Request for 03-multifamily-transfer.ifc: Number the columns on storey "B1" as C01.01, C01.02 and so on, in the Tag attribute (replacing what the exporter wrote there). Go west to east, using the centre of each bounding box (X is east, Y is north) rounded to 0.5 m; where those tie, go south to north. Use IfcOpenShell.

First a look at what the model holds.

```python
import ifcopenshell
import ifcopenshell.util.element
import ifcopenshell.util.placement

model = ifcopenshell.open("03-multifamily-transfer.ifc")
print(model.schema)
storey = next(s for s in model.by_type("IfcBuildingStorey") if s.Name == "B1")
columns = [e for e in ifcopenshell.util.element.get_decomposition(storey) if e.is_a("IfcColumn")]
for e in sorted(columns, key=lambda e: e.id()):
    origin = ifcopenshell.util.placement.get_local_placement(e.ObjectPlacement)[:3, 3]
    print(e.id(), e.Tag, e.Name, origin.round(2) + 0.0, sep=" | ")
```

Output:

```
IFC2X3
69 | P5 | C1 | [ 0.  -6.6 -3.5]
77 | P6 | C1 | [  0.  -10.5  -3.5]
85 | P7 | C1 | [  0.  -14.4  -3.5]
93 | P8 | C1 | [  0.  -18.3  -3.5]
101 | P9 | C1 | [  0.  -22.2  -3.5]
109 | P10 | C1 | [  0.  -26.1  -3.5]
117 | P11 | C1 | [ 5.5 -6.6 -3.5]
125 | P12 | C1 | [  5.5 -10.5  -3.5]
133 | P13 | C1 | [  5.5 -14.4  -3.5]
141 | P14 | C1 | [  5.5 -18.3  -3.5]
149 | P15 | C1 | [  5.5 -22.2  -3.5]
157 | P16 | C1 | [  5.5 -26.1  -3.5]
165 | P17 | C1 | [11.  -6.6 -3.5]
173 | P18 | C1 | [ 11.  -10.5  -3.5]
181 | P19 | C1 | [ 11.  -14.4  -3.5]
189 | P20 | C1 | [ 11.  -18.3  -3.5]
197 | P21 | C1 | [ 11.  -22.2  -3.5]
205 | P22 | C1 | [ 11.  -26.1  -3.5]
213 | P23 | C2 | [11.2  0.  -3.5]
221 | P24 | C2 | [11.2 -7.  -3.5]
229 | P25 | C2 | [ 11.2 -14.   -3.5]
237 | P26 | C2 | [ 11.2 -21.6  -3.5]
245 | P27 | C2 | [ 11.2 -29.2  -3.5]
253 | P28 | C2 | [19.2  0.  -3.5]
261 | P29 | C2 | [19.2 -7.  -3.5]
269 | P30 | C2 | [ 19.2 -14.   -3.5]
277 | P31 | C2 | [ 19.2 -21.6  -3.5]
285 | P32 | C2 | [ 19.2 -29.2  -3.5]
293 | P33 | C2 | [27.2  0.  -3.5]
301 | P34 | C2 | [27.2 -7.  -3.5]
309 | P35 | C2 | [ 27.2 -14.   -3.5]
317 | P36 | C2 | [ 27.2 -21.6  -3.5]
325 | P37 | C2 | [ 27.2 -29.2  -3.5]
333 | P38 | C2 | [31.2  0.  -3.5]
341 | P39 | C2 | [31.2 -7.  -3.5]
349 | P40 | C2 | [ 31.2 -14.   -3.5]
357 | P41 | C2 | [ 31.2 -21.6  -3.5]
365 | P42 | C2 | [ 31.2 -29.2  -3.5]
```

```python
import ifcopenshell
import ifcopenshell.geom
import ifcopenshell.util.element
import ifcopenshell.util.shape

model = ifcopenshell.open("03-multifamily-transfer.ifc")
settings = ifcopenshell.geom.settings()
settings.set("use-world-coords", True)


def centre(element):
    shape = ifcopenshell.geom.create_shape(settings, element)
    return ifcopenshell.util.shape.get_bbox_centroid(shape.geometry)


storey = next(s for s in model.by_type("IfcBuildingStorey") if s.Name == "B1")
columns = [e for e in ifcopenshell.util.element.get_decomposition(storey) if e.is_a("IfcColumn")]

# Insertion points can sit at a corner or the storey origin, so sort by the geometry (in metres).
centres = {e: centre(e) for e in columns}
columns.sort(key=lambda e: (round(centres[e][0] / 0.5), centres[e][1]))

for i, e in enumerate(columns, start=1):
    number = f"C01.{i:02d}"
    e.Tag = number
    print(e.id(), number)

model.write("03-multifamily-transfer_updated.ifc")
```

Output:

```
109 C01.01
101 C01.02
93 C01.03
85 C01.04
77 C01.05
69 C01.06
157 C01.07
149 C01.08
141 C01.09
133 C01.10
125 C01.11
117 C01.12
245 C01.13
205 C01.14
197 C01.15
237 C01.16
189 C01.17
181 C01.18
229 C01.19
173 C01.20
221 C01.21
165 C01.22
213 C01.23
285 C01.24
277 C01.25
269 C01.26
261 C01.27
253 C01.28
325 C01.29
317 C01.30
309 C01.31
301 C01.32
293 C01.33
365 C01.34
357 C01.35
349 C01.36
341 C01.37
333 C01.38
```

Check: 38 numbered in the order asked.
